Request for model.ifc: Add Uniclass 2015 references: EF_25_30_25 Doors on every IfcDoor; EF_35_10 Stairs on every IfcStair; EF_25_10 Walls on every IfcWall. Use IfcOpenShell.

First a look at what the model holds.

```python
import ifcopenshell

model = ifcopenshell.open("model.ifc")
print(model.schema)
print("classifications:", [c.Name for c in model.by_type("IfcClassification")])
for ifc_class in ("IfcDoor", "IfcRoof", "IfcStair", "IfcWall", "IfcWindow"):
    print(ifc_class, len(model.by_type(ifc_class)))
```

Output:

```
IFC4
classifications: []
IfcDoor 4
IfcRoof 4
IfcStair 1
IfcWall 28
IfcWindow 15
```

```python
import ifcopenshell
import ifcopenshell.api.classification

model = ifcopenshell.open("model.ifc")

system = ifcopenshell.api.classification.add_classification(model, classification="Uniclass 2015")

codes = {
    "IfcDoor": ("EF_25_30_25", "Doors"),
    "IfcStair": ("EF_35_10", "Stairs"),
    "IfcWall": ("EF_25_10", "Walls"),
}
for ifc_class, (code, name) in codes.items():
    products = model.by_type(ifc_class)
    ifcopenshell.api.classification.add_reference(
        model, products=products, classification=system, identification=code, name=name
    )
    print(code, len(products))

model.write("model_updated.ifc")
```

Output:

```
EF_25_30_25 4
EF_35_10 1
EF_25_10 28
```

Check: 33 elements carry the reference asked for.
